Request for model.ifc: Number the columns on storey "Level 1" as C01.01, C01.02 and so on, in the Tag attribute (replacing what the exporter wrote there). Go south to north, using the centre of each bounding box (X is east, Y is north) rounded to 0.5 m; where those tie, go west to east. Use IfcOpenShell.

First a look at what the model holds.

```python
import ifcopenshell
import ifcopenshell.util.element
import ifcopenshell.util.placement

model = ifcopenshell.open("model.ifc")
print(model.schema)
storey = next(s for s in model.by_type("IfcBuildingStorey") if s.Name == "Level 1")
columns = [e for e in ifcopenshell.util.element.get_decomposition(storey) if e.is_a("IfcColumn")]
for e in sorted(columns, key=lambda e: e.id()):
    origin = ifcopenshell.util.placement.get_local_placement(e.ObjectPlacement)[:3, 3]
    print(e.id(), e.Tag, e.Name, origin.round(2) + 0.0, sep=" | ")
```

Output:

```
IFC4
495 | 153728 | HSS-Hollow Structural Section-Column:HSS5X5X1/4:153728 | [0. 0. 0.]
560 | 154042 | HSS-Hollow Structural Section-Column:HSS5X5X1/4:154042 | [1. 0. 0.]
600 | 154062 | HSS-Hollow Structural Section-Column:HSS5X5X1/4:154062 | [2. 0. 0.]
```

```python
import ifcopenshell
import ifcopenshell.geom
import ifcopenshell.util.element
import ifcopenshell.util.shape

model = ifcopenshell.open("model.ifc")
settings = ifcopenshell.geom.settings()
settings.set("use-world-coords", True)


def centre(element):
    shape = ifcopenshell.geom.create_shape(settings, element)
    return ifcopenshell.util.shape.get_bbox_centroid(shape.geometry)


storey = next(s for s in model.by_type("IfcBuildingStorey") if s.Name == "Level 1")
columns = [e for e in ifcopenshell.util.element.get_decomposition(storey) if e.is_a("IfcColumn")]

# Insertion points can sit at a corner or the storey origin, so sort by the geometry (in metres).
centres = {e: centre(e) for e in columns}
columns.sort(key=lambda e: (round(centres[e][1] / 0.5), centres[e][0]))

for i, e in enumerate(columns, start=1):
    number = f"C01.{i:02d}"
    e.Tag = number
    print(e.id(), number)

model.write("model_rev.ifc")
```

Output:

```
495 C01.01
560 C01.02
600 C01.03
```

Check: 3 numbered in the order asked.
